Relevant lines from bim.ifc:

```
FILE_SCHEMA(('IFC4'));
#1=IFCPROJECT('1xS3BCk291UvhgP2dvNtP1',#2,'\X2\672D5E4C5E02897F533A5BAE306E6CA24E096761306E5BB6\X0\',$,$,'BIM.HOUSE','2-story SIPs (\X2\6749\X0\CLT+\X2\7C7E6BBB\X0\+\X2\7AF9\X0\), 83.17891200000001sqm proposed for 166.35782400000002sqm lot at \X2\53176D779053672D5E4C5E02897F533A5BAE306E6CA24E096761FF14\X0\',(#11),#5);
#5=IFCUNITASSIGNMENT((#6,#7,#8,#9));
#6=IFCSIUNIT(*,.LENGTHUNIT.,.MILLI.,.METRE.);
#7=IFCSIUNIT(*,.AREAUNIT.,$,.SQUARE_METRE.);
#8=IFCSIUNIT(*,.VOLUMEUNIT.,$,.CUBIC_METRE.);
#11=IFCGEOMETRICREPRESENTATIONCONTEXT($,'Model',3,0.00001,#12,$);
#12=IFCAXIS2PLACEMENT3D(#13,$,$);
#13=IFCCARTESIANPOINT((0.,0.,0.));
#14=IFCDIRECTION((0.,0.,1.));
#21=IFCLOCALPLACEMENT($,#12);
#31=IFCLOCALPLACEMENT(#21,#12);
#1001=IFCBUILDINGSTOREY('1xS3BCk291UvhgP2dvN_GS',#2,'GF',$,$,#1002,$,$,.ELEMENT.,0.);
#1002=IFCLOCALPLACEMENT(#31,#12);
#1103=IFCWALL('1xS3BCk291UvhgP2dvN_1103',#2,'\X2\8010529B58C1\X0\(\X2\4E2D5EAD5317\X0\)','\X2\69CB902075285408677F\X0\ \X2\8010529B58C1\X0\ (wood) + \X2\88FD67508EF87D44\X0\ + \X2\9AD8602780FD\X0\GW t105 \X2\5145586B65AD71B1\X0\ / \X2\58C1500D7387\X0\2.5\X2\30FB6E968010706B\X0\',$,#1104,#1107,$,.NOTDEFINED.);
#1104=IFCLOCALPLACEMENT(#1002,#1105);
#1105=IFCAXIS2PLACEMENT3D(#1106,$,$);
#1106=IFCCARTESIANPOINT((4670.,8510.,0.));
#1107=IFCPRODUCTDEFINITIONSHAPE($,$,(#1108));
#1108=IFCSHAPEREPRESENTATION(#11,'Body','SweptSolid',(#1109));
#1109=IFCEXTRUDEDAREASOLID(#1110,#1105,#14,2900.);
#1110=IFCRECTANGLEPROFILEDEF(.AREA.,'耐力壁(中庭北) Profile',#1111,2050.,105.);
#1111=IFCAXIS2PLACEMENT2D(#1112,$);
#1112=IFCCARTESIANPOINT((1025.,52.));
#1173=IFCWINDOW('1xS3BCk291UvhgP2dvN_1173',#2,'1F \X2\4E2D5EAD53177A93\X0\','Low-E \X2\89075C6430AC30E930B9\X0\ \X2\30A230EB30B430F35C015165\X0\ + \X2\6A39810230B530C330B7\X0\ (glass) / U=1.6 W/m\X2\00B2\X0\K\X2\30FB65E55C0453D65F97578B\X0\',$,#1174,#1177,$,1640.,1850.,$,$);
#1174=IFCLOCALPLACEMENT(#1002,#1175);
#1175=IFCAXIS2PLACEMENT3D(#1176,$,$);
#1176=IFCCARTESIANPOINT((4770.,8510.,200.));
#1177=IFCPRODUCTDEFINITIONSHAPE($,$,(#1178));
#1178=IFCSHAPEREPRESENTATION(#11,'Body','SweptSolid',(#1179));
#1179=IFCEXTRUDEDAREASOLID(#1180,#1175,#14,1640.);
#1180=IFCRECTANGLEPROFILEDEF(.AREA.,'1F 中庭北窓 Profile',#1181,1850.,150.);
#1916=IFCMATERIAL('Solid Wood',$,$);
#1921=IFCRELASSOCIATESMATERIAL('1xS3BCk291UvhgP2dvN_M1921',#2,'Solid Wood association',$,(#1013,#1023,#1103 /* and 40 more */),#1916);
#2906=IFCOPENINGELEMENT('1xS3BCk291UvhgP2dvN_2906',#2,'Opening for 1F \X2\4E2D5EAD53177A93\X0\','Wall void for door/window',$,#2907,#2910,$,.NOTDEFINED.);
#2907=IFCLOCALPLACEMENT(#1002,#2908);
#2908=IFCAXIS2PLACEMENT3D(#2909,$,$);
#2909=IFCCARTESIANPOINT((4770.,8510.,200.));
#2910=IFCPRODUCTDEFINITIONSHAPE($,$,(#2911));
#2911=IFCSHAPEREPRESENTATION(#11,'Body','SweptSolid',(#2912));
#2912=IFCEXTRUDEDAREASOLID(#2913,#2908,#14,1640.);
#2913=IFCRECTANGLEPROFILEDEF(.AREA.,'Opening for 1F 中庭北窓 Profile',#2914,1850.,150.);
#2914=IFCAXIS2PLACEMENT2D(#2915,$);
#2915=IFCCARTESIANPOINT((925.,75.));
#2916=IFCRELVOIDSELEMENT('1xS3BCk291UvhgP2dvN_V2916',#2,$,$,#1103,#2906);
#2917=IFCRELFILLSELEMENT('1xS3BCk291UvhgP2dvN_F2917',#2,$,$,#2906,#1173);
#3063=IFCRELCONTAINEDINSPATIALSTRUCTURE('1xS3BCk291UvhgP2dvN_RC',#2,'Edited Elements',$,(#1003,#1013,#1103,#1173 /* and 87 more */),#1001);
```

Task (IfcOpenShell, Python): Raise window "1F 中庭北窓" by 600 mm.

```python
import numpy as np
import ifcopenshell
import ifcopenshell.api.geometry
import ifcopenshell.util.placement
import ifcopenshell.util.unit

model = ifcopenshell.open("bim.ifc")
unit_scale = ifcopenshell.util.unit.calculate_unit_scale(model)

window = model.by_id(1173)
opening = window.FillsVoids[0].RelatingOpeningElement
dz = 600.0

shift = np.array([0.0, 0.0, dz])
# The window is not placed relative to its opening, so move both.
for product in (opening, window):
    matrix = ifcopenshell.util.placement.get_local_placement(product.ObjectPlacement)
    matrix[:3, 3] += shift
    ifcopenshell.api.geometry.edit_object_placement(model, product=product, matrix=matrix, is_si=False)

print(f"moved by {dz * unit_scale:+.3f} m")

model.write("bim_edited.ifc")
```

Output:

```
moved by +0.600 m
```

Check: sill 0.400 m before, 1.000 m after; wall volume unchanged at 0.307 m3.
